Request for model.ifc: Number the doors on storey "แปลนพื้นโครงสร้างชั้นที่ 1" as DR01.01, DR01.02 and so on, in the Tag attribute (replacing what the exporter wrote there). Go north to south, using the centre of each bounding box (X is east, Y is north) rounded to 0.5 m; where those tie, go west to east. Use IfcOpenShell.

First a look at what the model holds.

```python
import ifcopenshell
import ifcopenshell.util.element
import ifcopenshell.util.placement

model = ifcopenshell.open("model.ifc")
print(model.schema)
storey = next(s for s in model.by_type("IfcBuildingStorey") if s.Name == "แปลนพื้นโครงสร้างชั้นที่ 1")
doors = [e for e in ifcopenshell.util.element.get_decomposition(storey) if e.is_a("IfcDoor")]
for e in sorted(doors, key=lambda e: e.id()):
    origin = ifcopenshell.util.placement.get_local_placement(e.ObjectPlacement)[:3, 3]
    print(e.id(), e.Tag, e.Name, origin.round(2) + 0.0, sep=" | ")
```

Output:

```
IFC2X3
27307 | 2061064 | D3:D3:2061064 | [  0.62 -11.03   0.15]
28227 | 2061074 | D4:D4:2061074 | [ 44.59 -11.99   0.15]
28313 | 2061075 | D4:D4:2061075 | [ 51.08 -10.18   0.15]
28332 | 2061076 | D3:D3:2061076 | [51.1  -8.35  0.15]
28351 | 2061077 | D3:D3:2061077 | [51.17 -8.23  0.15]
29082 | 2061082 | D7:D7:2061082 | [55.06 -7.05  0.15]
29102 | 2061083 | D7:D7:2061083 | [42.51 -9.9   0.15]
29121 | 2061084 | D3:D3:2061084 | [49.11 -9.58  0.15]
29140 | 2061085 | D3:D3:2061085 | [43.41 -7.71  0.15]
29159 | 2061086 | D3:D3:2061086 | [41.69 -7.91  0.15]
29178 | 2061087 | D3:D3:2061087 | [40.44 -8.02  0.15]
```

```python
import ifcopenshell
import ifcopenshell.geom
import ifcopenshell.util.element
import ifcopenshell.util.shape

model = ifcopenshell.open("model.ifc")
settings = ifcopenshell.geom.settings()
settings.set("use-world-coords", True)


def centre(element):
    shape = ifcopenshell.geom.create_shape(settings, element)
    return ifcopenshell.util.shape.get_bbox_centroid(shape.geometry)


storey = next(s for s in model.by_type("IfcBuildingStorey") if s.Name == "แปลนพื้นโครงสร้างชั้นที่ 1")
doors = [e for e in ifcopenshell.util.element.get_decomposition(storey) if e.is_a("IfcDoor")]

# Insertion points can sit at a corner or the storey origin, so sort by the geometry (in metres).
centres = {e: centre(e) for e in doors}
doors.sort(key=lambda e: (-round(centres[e][1] / 0.5), centres[e][0]))

for i, e in enumerate(doors, start=1):
    number = f"DR01.{i:02d}"
    e.Tag = number
    print(e.id(), number)

model.write("model_rev.ifc")
```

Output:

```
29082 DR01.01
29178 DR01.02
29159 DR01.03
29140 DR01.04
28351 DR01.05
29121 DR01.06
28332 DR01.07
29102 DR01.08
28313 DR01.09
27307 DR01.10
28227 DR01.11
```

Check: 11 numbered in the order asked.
